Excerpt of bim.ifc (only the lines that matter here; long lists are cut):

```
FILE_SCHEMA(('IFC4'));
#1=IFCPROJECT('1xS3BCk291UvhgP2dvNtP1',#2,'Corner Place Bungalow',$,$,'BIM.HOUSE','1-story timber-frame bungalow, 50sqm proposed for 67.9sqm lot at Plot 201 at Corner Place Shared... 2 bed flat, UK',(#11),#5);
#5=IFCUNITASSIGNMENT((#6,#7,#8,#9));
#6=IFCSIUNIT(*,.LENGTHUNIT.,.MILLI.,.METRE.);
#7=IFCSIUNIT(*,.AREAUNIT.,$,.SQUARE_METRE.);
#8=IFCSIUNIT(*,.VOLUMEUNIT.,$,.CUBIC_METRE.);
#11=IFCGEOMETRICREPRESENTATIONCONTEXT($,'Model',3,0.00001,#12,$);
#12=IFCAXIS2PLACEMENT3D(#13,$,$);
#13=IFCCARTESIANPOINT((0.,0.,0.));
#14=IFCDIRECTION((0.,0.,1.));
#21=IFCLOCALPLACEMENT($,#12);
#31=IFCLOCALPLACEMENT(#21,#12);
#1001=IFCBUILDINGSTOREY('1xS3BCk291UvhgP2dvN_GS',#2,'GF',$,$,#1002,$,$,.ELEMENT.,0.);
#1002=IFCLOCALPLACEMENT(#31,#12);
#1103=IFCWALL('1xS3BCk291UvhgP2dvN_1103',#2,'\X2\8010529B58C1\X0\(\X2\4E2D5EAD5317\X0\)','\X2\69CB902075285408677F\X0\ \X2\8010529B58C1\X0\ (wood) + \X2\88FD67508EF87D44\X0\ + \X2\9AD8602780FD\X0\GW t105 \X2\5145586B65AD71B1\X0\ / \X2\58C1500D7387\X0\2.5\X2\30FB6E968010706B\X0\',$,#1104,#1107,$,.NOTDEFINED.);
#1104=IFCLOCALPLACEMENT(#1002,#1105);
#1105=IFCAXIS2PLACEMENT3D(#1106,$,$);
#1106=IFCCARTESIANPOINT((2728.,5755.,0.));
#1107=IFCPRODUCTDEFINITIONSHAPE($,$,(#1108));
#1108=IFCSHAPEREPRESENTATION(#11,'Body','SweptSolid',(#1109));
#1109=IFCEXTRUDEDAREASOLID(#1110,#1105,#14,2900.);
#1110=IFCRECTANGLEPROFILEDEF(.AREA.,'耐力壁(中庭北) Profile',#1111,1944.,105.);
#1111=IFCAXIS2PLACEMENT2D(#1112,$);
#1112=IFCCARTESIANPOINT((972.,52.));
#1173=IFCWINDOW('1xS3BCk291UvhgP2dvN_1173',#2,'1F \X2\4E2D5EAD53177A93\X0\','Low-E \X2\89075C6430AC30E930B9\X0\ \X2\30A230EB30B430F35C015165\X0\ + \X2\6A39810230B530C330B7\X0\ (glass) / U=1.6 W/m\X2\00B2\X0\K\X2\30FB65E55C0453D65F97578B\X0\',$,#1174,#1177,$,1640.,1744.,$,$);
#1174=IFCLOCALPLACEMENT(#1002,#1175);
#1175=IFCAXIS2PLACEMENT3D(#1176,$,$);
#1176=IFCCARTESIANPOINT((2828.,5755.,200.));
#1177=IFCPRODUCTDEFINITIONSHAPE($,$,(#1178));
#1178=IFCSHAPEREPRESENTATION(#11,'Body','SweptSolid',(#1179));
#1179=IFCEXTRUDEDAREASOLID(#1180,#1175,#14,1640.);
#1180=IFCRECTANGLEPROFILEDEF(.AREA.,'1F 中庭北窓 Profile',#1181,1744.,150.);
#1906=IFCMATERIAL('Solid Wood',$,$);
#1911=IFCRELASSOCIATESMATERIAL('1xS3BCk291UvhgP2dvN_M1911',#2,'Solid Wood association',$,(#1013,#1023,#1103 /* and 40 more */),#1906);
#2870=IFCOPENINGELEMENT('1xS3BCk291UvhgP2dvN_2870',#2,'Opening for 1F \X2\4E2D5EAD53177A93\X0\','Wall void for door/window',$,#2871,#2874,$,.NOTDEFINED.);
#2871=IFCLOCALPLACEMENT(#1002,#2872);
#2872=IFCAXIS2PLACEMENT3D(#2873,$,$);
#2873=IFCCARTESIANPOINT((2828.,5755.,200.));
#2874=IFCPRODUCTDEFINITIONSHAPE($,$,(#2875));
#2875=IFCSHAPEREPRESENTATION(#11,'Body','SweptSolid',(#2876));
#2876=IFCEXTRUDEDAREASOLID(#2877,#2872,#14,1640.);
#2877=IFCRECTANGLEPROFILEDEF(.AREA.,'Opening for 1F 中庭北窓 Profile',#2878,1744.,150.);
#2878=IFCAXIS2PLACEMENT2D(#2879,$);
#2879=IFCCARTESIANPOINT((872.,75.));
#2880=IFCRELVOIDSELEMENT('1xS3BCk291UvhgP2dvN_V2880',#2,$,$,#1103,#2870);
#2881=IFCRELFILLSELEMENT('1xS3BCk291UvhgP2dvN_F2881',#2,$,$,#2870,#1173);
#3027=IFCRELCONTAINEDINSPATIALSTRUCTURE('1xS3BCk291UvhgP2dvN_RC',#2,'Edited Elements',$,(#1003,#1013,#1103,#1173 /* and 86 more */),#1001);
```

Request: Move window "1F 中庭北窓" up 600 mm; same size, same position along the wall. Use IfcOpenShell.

```python
import numpy as np
import ifcopenshell
import ifcopenshell.api.geometry
import ifcopenshell.util.placement
import ifcopenshell.util.unit

model = ifcopenshell.open("bim.ifc")
unit_scale = ifcopenshell.util.unit.calculate_unit_scale(model)

window = model.by_guid("1xS3BCk291UvhgP2dvN_1173")
opening = window.FillsVoids[0].RelatingOpeningElement
dz = 600.0

shift = np.array([0.0, 0.0, dz])
# The window is not placed relative to its opening, so move both.
for product in (opening, window):
    matrix = ifcopenshell.util.placement.get_local_placement(product.ObjectPlacement)
    matrix[:3, 3] += shift
    ifcopenshell.api.geometry.edit_object_placement(model, product=product, matrix=matrix, is_si=False)

print(f"moved by {dz * unit_scale:+.3f} m")

model.write("bim_edited.ifc")
```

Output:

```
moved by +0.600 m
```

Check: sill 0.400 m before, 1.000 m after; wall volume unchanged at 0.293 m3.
